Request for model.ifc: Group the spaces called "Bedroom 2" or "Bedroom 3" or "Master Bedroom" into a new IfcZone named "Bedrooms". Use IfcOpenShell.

First a look at what the model holds.

```python
import ifcopenshell

model = ifcopenshell.open("model.ifc")
print(model.schema)
seen = {}
for space in model.by_type("IfcSpace"):
    seen[space.LongName] = seen.get(space.LongName, 0) + 1
for name, count in sorted(seen.items(), key=str):
    print(count, "x", name)
print("zones:", [z.Name for z in model.by_type("IfcZone")][:20])
```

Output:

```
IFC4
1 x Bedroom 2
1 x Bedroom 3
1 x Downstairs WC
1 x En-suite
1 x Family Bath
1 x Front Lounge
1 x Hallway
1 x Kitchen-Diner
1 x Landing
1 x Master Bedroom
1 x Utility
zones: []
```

```python
import ifcopenshell
import ifcopenshell.api.group
import ifcopenshell.api.root

model = ifcopenshell.open("model.ifc")

names = {"Bedroom 2", "Bedroom 3", "Master Bedroom"}
spaces = [s for s in model.by_type("IfcSpace") if s.LongName in names]

zone = ifcopenshell.api.root.create_entity(model, ifc_class="IfcZone", name="Bedrooms")
ifcopenshell.api.group.assign_group(model, products=spaces, group=zone)
print(len(spaces), "spaces in", zone.Name)

model.write("model_edited.ifc")
```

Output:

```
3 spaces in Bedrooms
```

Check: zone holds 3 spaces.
